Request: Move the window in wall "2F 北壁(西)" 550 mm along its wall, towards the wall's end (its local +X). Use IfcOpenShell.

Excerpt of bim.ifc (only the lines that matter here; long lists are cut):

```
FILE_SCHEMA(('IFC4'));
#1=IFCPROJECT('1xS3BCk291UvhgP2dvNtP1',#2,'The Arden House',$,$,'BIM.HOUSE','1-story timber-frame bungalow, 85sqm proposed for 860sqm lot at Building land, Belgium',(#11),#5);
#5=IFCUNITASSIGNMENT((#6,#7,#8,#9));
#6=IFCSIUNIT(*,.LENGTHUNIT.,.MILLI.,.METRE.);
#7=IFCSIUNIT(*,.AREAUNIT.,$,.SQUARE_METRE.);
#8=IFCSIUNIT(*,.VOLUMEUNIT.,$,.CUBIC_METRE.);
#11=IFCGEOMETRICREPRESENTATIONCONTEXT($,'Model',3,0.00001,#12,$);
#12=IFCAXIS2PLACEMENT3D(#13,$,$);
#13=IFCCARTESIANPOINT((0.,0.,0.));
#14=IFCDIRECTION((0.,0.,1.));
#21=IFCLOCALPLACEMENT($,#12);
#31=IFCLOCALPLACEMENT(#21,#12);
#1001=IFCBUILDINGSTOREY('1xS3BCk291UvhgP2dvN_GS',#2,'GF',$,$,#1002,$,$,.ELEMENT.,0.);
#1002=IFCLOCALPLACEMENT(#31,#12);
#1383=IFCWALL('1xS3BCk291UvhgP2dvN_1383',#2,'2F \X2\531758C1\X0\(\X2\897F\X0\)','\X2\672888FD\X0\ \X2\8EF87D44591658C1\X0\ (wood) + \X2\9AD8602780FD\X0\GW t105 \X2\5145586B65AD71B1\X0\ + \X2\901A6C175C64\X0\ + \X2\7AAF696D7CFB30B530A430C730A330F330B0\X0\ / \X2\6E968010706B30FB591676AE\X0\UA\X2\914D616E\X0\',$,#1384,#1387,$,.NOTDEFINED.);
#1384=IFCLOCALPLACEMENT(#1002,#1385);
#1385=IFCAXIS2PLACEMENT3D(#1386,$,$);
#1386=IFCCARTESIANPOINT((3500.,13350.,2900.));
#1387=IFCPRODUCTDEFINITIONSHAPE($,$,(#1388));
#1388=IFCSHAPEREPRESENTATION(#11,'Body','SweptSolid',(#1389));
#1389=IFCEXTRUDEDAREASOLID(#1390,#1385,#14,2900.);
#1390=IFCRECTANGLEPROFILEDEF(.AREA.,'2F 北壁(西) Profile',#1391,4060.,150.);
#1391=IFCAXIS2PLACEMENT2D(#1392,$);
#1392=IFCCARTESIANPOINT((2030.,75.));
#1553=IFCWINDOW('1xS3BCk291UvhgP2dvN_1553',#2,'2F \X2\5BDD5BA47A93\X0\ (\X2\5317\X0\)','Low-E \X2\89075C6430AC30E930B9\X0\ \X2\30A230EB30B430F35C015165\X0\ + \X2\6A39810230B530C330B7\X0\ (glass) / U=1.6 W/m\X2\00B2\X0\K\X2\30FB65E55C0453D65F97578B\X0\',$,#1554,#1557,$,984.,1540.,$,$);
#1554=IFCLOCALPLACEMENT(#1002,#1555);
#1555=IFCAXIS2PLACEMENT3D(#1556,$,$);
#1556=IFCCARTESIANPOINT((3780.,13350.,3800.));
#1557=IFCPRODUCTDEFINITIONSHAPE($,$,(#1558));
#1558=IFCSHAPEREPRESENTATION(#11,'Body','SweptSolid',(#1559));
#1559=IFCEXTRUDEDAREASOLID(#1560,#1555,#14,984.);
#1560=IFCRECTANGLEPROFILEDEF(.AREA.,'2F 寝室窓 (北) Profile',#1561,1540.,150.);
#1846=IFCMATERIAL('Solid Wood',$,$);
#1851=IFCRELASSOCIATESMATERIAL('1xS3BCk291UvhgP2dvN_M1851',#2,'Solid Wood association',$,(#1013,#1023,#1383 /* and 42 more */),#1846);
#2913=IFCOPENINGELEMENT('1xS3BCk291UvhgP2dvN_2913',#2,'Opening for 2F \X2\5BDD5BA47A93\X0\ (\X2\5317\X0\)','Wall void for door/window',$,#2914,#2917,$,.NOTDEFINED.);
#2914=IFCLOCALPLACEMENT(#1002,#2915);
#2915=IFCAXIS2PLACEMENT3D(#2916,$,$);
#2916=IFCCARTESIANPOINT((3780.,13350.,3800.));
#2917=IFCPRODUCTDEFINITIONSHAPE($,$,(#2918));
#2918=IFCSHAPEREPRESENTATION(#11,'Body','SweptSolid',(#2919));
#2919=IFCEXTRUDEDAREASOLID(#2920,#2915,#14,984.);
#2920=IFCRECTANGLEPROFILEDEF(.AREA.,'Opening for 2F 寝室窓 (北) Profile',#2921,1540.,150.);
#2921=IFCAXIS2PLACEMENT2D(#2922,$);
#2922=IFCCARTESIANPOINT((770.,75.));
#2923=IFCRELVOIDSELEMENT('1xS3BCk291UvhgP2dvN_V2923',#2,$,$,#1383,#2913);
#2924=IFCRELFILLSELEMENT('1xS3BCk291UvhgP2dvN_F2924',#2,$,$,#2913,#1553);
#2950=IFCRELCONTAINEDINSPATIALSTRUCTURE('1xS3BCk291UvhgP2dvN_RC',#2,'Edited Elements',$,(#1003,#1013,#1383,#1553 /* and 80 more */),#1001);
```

```python
import ifcopenshell
import ifcopenshell.api.geometry
import ifcopenshell.util.placement
import ifcopenshell.util.unit

model = ifcopenshell.open("bim.ifc")
unit_scale = ifcopenshell.util.unit.calculate_unit_scale(model)

window = model.by_guid("1xS3BCk291UvhgP2dvN_1553")
opening = window.FillsVoids[0].RelatingOpeningElement
wall = opening.VoidsElements[0].RelatingBuildingElement

wall_matrix = ifcopenshell.util.placement.get_local_placement(wall.ObjectPlacement)
shift = wall_matrix[:3, 0] * 0.55 / unit_scale
before = ifcopenshell.util.placement.get_local_placement(window.ObjectPlacement)[:3, 3].copy()

# The window is not placed relative to its opening, so move both.
for product in (opening, window):
    matrix = ifcopenshell.util.placement.get_local_placement(product.ObjectPlacement)
    matrix[:3, 3] += shift
    ifcopenshell.api.geometry.edit_object_placement(model, product=product, matrix=matrix, is_si=False)

after = ifcopenshell.util.placement.get_local_placement(window.ObjectPlacement)[:3, 3]
print("window moved by", (after - before).round(3) + 0.0)

model.write("bim_updated.ifc")
```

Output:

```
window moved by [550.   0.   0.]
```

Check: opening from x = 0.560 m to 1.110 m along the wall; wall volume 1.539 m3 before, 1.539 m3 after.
